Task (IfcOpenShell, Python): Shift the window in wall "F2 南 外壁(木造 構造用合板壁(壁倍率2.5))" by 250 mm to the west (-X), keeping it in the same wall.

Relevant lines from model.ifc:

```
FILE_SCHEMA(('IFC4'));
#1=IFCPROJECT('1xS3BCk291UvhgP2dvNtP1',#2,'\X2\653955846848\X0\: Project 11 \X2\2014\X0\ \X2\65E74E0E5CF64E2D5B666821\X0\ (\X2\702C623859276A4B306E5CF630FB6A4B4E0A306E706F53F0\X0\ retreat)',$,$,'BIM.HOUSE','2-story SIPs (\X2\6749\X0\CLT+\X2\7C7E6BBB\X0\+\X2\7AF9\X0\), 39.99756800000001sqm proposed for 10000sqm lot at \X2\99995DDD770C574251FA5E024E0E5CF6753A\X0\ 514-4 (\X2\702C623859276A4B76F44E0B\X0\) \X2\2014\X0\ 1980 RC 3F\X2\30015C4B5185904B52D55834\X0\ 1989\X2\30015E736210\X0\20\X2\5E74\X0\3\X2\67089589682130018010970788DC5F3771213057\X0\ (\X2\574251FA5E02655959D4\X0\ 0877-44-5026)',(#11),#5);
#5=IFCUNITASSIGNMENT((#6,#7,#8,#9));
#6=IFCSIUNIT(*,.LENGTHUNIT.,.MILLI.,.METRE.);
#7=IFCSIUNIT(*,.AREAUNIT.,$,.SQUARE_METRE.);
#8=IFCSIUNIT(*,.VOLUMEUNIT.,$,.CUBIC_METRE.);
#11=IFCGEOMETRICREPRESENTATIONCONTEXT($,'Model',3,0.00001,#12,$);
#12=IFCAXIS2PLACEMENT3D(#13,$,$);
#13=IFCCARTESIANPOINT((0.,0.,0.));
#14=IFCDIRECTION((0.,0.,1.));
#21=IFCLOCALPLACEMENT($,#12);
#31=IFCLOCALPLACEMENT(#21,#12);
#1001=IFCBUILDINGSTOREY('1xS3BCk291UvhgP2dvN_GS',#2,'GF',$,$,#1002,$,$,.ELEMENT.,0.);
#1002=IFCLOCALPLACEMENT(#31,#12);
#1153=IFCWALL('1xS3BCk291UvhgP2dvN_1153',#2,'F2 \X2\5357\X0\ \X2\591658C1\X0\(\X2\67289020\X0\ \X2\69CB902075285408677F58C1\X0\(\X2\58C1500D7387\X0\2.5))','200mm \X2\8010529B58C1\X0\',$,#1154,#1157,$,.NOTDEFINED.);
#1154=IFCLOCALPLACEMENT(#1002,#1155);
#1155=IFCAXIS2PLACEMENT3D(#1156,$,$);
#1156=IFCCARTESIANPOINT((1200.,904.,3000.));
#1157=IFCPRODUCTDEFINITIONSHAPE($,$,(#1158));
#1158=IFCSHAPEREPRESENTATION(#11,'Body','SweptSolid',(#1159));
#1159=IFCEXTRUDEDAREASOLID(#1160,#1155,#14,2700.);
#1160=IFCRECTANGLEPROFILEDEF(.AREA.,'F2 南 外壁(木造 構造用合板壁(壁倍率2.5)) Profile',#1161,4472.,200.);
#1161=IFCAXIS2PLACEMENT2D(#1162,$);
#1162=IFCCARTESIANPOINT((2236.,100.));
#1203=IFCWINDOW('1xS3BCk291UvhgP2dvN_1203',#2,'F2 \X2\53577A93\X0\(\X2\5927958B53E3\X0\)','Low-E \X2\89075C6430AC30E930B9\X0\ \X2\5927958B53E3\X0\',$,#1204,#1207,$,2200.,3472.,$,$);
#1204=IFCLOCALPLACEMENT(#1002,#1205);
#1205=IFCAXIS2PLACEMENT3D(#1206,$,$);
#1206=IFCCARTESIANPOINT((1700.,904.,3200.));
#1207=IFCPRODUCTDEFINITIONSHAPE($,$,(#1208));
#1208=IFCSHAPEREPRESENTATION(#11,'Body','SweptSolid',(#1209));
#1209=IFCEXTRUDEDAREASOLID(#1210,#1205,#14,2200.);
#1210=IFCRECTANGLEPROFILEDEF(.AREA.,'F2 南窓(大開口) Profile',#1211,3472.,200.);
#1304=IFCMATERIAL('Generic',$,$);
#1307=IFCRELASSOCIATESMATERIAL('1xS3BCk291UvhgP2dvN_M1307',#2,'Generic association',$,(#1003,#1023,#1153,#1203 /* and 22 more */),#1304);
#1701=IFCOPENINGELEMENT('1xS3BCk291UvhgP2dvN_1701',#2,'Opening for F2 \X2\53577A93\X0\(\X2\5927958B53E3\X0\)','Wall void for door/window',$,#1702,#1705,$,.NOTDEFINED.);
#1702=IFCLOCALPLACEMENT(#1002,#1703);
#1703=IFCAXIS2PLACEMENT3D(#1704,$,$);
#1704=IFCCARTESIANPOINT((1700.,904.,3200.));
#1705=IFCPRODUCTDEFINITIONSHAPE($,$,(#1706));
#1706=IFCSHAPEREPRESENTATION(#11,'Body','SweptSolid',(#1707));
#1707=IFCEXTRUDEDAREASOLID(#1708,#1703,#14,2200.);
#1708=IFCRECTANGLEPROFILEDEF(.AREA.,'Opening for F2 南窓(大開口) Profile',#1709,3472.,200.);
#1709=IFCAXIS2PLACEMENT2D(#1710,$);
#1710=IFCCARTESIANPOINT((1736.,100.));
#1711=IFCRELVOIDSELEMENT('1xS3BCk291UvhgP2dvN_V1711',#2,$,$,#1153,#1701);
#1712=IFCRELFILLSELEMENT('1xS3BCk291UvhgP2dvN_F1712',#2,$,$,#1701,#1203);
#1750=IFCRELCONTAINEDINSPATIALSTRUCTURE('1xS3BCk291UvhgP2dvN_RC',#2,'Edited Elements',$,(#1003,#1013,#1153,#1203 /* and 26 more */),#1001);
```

```python
import ifcopenshell
import ifcopenshell.api.geometry
import ifcopenshell.util.placement

model = ifcopenshell.open("model.ifc")

window = model.by_guid("1xS3BCk291UvhgP2dvN_1203")
opening = window.FillsVoids[0].RelatingOpeningElement
wall = opening.VoidsElements[0].RelatingBuildingElement

wall_matrix = ifcopenshell.util.placement.get_local_placement(wall.ObjectPlacement)
shift = wall_matrix[:3, 0] * -250.0
before = ifcopenshell.util.placement.get_local_placement(window.ObjectPlacement)[:3, 3].copy()

# The window is not placed relative to its opening, so move both.
for product in (opening, window):
    matrix = ifcopenshell.util.placement.get_local_placement(product.ObjectPlacement)
    matrix[:3, 3] += shift
    ifcopenshell.api.geometry.edit_object_placement(model, product=product, matrix=matrix, is_si=False)

after = ifcopenshell.util.placement.get_local_placement(window.ObjectPlacement)[:3, 3]
print("window moved by", (after - before).round(3) + 0.0)

model.write("model_rev.ifc")
```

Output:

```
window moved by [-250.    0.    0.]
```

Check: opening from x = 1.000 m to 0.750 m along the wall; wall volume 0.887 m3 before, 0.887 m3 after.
